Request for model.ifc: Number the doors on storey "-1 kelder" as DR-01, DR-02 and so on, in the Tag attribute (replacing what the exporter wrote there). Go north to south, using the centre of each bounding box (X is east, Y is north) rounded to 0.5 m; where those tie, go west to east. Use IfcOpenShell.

First a look at what the model holds.

```python
import ifcopenshell
import ifcopenshell.util.element
import ifcopenshell.util.placement

model = ifcopenshell.open("model.ifc")
print(model.schema)
storey = next(s for s in model.by_type("IfcBuildingStorey") if s.Name == "-1 kelder")
doors = [e for e in ifcopenshell.util.element.get_decomposition(storey) if e.is_a("IfcDoor")]
for e in sorted(doors, key=lambda e: e.id()):
    origin = ifcopenshell.util.placement.get_local_placement(e.ObjectPlacement)[:3, 3]
    print(e.id(), e.Tag, e.Name, origin.round(2) + 0.0, sep=" | ")
```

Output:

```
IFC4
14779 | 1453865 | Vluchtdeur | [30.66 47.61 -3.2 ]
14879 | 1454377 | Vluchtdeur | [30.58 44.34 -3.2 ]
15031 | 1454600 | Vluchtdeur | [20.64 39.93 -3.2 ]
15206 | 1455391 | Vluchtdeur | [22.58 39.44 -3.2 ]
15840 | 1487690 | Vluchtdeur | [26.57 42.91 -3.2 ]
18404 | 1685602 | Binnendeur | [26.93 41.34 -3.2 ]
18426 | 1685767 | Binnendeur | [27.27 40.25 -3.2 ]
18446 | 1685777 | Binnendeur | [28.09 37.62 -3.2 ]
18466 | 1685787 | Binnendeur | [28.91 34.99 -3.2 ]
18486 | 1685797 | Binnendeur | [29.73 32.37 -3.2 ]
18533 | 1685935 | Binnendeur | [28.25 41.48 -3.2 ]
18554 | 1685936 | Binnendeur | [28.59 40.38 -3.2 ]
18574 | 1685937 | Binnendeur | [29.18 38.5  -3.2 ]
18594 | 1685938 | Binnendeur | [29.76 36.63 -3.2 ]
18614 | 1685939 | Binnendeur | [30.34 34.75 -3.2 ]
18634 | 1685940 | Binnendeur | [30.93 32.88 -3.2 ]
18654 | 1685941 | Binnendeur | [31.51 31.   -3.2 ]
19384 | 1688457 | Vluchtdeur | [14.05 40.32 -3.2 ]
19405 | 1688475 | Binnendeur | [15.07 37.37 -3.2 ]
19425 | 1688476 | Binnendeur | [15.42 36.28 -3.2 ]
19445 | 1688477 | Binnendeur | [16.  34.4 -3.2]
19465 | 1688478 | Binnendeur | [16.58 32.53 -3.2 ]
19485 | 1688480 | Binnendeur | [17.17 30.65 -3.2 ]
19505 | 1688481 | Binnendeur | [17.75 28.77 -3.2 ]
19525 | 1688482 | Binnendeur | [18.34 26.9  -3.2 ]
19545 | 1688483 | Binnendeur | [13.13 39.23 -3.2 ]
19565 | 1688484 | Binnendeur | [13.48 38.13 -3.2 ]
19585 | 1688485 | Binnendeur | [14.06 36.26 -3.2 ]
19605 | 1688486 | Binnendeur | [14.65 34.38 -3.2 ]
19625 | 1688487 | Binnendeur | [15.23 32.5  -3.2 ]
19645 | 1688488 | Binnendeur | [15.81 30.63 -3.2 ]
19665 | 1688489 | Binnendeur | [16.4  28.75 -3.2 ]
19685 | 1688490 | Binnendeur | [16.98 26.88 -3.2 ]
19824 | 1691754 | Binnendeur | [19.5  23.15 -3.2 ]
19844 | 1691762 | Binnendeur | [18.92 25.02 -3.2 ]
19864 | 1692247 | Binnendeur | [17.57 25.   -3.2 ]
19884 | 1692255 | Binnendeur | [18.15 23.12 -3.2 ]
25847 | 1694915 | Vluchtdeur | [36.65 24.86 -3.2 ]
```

```python
import ifcopenshell
import ifcopenshell.geom
import ifcopenshell.util.element
import ifcopenshell.util.shape

model = ifcopenshell.open("model.ifc")
settings = ifcopenshell.geom.settings()
settings.set("use-world-coords", True)


def centre(element):
    shape = ifcopenshell.geom.create_shape(settings, element)
    return ifcopenshell.util.shape.get_bbox_centroid(shape.geometry)


storey = next(s for s in model.by_type("IfcBuildingStorey") if s.Name == "-1 kelder")
doors = [e for e in ifcopenshell.util.element.get_decomposition(storey) if e.is_a("IfcDoor")]

# Insertion points can sit at a corner or the storey origin, so sort by the geometry (in metres).
centres = {e: centre(e) for e in doors}
doors.sort(key=lambda e: (-round(centres[e][1] / 0.5), centres[e][0]))

for i, e in enumerate(doors, start=1):
    number = f"DR-{i:02d}"
    e.Tag = number
    print(e.id(), number)

model.write("model_v2.ifc")
```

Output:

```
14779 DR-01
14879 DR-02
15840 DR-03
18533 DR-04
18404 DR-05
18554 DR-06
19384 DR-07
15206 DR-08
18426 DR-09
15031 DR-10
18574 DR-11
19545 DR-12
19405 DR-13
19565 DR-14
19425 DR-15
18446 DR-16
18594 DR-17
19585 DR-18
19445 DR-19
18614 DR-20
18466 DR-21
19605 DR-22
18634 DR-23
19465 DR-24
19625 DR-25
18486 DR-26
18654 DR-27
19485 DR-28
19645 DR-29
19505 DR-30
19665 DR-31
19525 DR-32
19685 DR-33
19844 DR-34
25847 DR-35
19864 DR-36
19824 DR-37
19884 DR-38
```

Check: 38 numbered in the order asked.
